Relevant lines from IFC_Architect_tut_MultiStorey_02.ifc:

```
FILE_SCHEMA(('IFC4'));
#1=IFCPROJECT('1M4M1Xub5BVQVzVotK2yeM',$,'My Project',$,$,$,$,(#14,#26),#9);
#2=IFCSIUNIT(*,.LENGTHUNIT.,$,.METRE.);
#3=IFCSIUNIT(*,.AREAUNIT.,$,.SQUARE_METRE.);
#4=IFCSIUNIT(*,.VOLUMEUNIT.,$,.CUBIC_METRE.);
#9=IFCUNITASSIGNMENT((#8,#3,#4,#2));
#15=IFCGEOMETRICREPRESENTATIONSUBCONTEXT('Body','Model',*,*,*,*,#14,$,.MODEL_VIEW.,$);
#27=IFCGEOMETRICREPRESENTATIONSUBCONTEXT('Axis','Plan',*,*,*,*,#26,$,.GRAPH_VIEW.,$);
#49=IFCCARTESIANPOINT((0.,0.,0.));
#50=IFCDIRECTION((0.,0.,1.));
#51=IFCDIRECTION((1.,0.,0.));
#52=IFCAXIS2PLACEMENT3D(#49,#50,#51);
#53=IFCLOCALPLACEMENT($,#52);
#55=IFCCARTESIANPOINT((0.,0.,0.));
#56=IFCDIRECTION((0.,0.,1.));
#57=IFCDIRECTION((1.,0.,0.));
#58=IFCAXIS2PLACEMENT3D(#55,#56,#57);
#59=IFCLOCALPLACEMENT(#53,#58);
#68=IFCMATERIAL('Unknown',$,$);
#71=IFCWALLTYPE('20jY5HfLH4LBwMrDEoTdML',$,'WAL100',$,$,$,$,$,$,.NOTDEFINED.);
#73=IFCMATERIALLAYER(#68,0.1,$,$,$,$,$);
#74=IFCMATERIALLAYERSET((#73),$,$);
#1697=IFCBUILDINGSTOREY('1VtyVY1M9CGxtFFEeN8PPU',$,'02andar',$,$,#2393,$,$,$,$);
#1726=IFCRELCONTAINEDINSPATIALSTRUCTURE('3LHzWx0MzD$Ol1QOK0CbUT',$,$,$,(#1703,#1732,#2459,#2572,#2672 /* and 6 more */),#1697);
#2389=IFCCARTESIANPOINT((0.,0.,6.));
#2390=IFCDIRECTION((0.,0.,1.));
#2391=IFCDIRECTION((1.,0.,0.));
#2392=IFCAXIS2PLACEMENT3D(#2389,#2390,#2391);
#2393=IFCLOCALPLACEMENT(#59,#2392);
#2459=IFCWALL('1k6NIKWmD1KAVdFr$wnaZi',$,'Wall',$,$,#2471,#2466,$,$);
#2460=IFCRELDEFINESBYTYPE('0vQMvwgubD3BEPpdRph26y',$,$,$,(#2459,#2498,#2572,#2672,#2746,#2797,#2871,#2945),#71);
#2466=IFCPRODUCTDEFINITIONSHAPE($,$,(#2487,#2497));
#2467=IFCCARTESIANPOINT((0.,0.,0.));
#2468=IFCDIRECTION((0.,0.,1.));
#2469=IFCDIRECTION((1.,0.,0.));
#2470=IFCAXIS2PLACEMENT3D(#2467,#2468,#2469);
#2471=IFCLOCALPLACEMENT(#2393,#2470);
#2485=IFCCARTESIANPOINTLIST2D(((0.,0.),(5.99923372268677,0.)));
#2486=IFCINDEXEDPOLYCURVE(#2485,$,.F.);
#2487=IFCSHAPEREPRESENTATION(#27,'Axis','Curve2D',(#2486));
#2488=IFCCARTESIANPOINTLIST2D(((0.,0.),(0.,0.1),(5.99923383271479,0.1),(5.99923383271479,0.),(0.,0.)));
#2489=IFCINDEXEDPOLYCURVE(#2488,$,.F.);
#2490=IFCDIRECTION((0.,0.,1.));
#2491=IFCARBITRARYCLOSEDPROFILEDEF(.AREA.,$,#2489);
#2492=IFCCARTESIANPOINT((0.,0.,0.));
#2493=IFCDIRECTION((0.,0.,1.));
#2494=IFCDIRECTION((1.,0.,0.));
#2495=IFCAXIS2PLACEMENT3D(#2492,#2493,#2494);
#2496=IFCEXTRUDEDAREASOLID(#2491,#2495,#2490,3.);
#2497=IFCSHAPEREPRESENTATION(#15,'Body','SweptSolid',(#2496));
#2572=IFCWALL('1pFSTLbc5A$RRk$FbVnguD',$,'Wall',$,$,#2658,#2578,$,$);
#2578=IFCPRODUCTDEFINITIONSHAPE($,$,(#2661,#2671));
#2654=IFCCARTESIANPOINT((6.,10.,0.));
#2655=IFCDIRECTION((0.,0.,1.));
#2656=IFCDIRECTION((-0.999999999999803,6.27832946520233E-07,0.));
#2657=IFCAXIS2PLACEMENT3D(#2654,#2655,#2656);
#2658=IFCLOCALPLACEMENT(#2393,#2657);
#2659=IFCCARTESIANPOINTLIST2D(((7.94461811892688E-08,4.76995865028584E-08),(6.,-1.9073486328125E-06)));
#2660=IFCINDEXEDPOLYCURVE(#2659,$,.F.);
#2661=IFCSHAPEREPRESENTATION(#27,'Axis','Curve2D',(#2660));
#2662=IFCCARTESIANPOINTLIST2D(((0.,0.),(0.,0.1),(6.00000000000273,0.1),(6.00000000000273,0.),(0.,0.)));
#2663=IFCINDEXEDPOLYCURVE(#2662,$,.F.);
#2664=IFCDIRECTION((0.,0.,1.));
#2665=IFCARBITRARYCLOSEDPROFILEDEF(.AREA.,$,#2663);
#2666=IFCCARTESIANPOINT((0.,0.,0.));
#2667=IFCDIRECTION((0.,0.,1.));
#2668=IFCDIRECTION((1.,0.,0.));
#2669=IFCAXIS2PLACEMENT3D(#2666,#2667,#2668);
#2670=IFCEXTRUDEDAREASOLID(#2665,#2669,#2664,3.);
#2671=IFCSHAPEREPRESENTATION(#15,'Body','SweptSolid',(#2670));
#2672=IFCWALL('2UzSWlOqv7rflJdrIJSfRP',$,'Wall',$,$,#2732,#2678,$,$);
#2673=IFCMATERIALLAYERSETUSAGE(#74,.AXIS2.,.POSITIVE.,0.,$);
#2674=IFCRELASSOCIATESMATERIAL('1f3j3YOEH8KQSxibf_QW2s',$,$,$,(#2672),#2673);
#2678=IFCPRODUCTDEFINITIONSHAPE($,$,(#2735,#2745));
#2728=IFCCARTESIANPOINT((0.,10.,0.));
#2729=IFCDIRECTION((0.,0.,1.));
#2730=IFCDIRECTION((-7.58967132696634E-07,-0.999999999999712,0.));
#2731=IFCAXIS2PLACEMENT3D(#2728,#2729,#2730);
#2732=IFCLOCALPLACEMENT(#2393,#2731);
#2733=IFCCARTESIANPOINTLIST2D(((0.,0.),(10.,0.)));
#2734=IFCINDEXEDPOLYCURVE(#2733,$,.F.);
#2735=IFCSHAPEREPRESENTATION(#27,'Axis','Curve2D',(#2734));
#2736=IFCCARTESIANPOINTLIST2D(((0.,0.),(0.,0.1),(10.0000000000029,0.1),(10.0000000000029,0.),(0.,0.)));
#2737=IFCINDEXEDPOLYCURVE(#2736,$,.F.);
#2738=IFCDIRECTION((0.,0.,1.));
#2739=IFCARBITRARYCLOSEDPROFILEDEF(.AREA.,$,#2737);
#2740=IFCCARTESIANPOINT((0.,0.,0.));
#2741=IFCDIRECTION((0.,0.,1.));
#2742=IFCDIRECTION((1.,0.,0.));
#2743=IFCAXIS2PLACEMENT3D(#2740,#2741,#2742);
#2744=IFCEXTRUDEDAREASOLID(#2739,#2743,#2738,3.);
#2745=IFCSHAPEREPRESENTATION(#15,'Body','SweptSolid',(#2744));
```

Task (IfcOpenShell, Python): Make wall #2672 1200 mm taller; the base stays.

```python
import ifcopenshell
import ifcopenshell.geom
import ifcopenshell.util.representation
import ifcopenshell.util.shape
import ifcopenshell.util.unit

model = ifcopenshell.open("IFC_Architect_tut_MultiStorey_02.ifc")
unit_scale = ifcopenshell.util.unit.calculate_unit_scale(model)
settings = ifcopenshell.geom.settings()


def volume(element):
    """Net volume in cubic metres, openings subtracted."""
    shape = ifcopenshell.geom.create_shape(settings, element)
    return ifcopenshell.util.shape.get_volume(shape.geometry)


wall = model.by_id(2672)
before = volume(wall)

body = ifcopenshell.util.representation.get_representation(wall, "Model", "Body")
solid = body.Items[0]
old_height = solid.Depth
solid.Depth += 1.2 / unit_scale
after = volume(wall)

print(f"height {old_height:g} -> {solid.Depth:g}, volume {before:.3f} -> {after:.3f} m3")

model.write("IFC_Architect_tut_MultiStorey_02_updated.ifc")
```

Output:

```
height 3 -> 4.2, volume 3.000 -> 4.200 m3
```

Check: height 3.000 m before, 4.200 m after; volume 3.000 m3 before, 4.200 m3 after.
